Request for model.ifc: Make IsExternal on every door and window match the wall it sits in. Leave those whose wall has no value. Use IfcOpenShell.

First a look at what the model holds.

```python
import ifcopenshell
import ifcopenshell.util.element

model = ifcopenshell.open("model.ifc")
print(model.schema)
seen = {}
for e in model.by_type("IfcDoor") + model.by_type("IfcWindow"):
    if not e.FillsVoids:
        continue
    host = e.FillsVoids[0].RelatingOpeningElement.VoidsElements[0].RelatingBuildingElement
    own = ifcopenshell.util.element.get_pset(e, f"Pset_{e.is_a()[3:].removesuffix('StandardCase')}Common", "IsExternal")
    wall = ifcopenshell.util.element.get_pset(host, "Pset_WallCommon", "IsExternal")
    seen[e.is_a(), own, wall] = seen.get((e.is_a(), own, wall), 0) + 1
for (cls, own, wall), count in sorted(seen.items(), key=str):
    print(count, cls, "IsExternal:", own, "| host wall:", wall)
```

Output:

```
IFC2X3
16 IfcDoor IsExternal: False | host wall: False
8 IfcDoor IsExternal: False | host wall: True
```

```python
import ifcopenshell
import ifcopenshell.api.pset
import ifcopenshell.util.element

model = ifcopenshell.open("model.ifc")

count = 0
for ifc_class, pset_name in (("IfcDoor", "Pset_DoorCommon"), ("IfcWindow", "Pset_WindowCommon")):
    for e in model.by_type(ifc_class):
        if not e.FillsVoids:
            continue
        host = e.FillsVoids[0].RelatingOpeningElement.VoidsElements[0].RelatingBuildingElement
        external = ifcopenshell.util.element.get_pset(host, "Pset_WallCommon", "IsExternal")
        if external is None or ifcopenshell.util.element.get_pset(e, pset_name, "IsExternal") == external:
            continue
        pset = ifcopenshell.api.pset.add_pset(model, product=e, name=pset_name)
        ifcopenshell.api.pset.edit_pset(model, pset=pset, properties={"IsExternal": external})
        count += 1

print(count, "updated")

model.write("model_rev.ifc")
```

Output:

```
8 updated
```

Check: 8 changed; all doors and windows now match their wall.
